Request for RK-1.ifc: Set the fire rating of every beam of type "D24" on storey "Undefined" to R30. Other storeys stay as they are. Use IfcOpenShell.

First a look at what the model holds.

```python
import ifcopenshell
import ifcopenshell.util.element

model = ifcopenshell.open("RK-1.ifc")
print(model.schema)
storey = next(s for s in model.by_type("IfcBuildingStorey") if s.Name == "Undefined")
beams = [e for e in ifcopenshell.util.element.get_decomposition(storey) if e.is_a("IfcBeam")]
seen = {}
for e in beams:
    element_type = ifcopenshell.util.element.get_type(e)
    key = (element_type.Name if element_type != e and element_type else None, ifcopenshell.util.element.get_pset(e, "Pset_BeamCommon", "FireRating"))
    seen[key] = seen.get(key, 0) + 1
for (name, value), count in sorted(seen.items(), key=str):
    print(count, "x", name, "|", value)
```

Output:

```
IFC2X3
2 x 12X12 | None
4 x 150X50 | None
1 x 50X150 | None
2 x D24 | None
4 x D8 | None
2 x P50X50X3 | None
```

```python
import ifcopenshell
import ifcopenshell.api.pset
import ifcopenshell.util.element

model = ifcopenshell.open("RK-1.ifc")

storey = next(s for s in model.by_type("IfcBuildingStorey") if s.Name == "Undefined")
beams = [e for e in ifcopenshell.util.element.get_decomposition(storey) if e.is_a("IfcBeam")]

count = 0
for e in beams:
    element_type = ifcopenshell.util.element.get_type(e)
    if element_type in (None, e) or element_type.Name != "D24":
        continue
    found = ifcopenshell.util.element.get_pset(e, "Pset_BeamCommon", should_inherit=False)
    if found:
        pset = model.by_id(found["id"])
        if len(ifcopenshell.util.element.get_elements_by_pset(pset)) > 1:
            pset = ifcopenshell.api.pset.unshare_pset(model, products=[e], pset=pset)[0]
    else:
        pset = ifcopenshell.api.pset.add_pset(model, product=e, name="Pset_BeamCommon")
    ifcopenshell.api.pset.edit_pset(model, pset=pset, properties={"FireRating": "R30"})
    count += 1

print(count, "beams updated")

model.write("RK-1_edited.ifc")
```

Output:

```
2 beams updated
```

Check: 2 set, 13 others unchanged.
